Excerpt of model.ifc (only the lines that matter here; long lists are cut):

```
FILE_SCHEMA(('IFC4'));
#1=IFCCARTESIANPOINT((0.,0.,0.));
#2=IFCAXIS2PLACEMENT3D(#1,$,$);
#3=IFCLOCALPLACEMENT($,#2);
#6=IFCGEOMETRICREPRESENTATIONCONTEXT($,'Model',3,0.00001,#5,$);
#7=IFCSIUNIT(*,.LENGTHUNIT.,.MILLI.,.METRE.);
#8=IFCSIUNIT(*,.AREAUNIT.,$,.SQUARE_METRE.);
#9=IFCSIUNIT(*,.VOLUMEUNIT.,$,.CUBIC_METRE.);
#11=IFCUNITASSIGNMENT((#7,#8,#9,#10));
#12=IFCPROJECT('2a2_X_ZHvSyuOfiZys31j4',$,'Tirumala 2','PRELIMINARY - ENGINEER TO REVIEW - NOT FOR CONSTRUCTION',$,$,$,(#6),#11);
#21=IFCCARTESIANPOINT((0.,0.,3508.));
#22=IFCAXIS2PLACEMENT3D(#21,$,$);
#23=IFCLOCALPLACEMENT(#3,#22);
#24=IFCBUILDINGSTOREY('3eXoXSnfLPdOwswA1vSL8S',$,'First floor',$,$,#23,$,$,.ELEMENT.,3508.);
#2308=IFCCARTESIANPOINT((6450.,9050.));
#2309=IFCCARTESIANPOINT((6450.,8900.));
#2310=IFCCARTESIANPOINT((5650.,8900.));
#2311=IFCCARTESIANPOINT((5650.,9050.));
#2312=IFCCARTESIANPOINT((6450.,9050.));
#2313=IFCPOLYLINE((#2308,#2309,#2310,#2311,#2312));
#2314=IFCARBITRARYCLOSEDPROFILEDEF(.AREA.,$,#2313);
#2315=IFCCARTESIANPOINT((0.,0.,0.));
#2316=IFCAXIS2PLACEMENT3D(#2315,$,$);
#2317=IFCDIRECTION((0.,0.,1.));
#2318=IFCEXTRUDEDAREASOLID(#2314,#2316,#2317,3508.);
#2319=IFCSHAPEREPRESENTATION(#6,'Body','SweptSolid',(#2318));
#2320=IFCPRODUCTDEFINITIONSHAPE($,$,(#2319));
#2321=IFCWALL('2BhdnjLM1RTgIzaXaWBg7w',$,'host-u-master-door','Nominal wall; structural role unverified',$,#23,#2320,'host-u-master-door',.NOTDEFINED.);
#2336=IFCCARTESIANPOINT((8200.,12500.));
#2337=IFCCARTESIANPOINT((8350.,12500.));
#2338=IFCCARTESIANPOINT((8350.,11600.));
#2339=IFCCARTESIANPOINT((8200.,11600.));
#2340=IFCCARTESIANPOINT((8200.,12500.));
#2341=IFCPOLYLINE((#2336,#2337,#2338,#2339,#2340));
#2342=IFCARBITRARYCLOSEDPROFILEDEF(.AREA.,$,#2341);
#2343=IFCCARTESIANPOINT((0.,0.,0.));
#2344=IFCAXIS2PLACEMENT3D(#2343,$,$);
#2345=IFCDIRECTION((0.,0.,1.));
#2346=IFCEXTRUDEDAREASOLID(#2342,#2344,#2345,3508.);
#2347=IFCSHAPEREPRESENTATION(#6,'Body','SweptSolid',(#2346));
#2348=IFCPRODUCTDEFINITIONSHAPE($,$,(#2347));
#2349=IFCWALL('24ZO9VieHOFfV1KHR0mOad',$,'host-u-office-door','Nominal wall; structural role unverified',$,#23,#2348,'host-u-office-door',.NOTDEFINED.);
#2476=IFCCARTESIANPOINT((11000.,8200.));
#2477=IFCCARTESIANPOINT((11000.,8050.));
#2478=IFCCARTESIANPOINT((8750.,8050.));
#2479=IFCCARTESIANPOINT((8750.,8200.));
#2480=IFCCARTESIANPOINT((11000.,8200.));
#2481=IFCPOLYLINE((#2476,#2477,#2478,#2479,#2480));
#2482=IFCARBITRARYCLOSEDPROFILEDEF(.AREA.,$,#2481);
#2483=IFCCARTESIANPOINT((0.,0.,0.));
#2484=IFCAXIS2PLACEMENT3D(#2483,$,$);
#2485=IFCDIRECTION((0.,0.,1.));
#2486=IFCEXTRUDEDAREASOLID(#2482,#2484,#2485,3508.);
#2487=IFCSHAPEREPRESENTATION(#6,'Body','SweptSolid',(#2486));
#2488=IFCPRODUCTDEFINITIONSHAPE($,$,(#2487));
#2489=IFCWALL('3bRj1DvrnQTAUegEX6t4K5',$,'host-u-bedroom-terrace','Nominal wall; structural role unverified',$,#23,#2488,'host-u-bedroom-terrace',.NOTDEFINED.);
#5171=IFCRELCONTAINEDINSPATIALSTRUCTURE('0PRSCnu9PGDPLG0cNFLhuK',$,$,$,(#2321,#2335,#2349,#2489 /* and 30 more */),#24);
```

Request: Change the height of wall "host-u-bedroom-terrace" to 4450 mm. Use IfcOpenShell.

```python
import ifcopenshell
import ifcopenshell.geom
import ifcopenshell.util.shape
import ifcopenshell.util.unit

model = ifcopenshell.open("model.ifc")
unit_scale = ifcopenshell.util.unit.calculate_unit_scale(model)
settings = ifcopenshell.geom.settings()


def volume(element):
    """Net volume in cubic metres, openings subtracted."""
    shape = ifcopenshell.geom.create_shape(settings, element)
    return ifcopenshell.util.shape.get_volume(shape.geometry)


wall = model.by_id(2489)
before = volume(wall)

body = next(r for r in wall.Representation.Representations if r.RepresentationIdentifier == "Body")
solid = body.Items[0]
old_height = solid.Depth
solid.Depth = 4.45 / unit_scale
after = volume(wall)

print(f"height {old_height:g} -> {solid.Depth:g}, volume {before:.3f} -> {after:.3f} m3")

model.write("model_v2.ifc")
```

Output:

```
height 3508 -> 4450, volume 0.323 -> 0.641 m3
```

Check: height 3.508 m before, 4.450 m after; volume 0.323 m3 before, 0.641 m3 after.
